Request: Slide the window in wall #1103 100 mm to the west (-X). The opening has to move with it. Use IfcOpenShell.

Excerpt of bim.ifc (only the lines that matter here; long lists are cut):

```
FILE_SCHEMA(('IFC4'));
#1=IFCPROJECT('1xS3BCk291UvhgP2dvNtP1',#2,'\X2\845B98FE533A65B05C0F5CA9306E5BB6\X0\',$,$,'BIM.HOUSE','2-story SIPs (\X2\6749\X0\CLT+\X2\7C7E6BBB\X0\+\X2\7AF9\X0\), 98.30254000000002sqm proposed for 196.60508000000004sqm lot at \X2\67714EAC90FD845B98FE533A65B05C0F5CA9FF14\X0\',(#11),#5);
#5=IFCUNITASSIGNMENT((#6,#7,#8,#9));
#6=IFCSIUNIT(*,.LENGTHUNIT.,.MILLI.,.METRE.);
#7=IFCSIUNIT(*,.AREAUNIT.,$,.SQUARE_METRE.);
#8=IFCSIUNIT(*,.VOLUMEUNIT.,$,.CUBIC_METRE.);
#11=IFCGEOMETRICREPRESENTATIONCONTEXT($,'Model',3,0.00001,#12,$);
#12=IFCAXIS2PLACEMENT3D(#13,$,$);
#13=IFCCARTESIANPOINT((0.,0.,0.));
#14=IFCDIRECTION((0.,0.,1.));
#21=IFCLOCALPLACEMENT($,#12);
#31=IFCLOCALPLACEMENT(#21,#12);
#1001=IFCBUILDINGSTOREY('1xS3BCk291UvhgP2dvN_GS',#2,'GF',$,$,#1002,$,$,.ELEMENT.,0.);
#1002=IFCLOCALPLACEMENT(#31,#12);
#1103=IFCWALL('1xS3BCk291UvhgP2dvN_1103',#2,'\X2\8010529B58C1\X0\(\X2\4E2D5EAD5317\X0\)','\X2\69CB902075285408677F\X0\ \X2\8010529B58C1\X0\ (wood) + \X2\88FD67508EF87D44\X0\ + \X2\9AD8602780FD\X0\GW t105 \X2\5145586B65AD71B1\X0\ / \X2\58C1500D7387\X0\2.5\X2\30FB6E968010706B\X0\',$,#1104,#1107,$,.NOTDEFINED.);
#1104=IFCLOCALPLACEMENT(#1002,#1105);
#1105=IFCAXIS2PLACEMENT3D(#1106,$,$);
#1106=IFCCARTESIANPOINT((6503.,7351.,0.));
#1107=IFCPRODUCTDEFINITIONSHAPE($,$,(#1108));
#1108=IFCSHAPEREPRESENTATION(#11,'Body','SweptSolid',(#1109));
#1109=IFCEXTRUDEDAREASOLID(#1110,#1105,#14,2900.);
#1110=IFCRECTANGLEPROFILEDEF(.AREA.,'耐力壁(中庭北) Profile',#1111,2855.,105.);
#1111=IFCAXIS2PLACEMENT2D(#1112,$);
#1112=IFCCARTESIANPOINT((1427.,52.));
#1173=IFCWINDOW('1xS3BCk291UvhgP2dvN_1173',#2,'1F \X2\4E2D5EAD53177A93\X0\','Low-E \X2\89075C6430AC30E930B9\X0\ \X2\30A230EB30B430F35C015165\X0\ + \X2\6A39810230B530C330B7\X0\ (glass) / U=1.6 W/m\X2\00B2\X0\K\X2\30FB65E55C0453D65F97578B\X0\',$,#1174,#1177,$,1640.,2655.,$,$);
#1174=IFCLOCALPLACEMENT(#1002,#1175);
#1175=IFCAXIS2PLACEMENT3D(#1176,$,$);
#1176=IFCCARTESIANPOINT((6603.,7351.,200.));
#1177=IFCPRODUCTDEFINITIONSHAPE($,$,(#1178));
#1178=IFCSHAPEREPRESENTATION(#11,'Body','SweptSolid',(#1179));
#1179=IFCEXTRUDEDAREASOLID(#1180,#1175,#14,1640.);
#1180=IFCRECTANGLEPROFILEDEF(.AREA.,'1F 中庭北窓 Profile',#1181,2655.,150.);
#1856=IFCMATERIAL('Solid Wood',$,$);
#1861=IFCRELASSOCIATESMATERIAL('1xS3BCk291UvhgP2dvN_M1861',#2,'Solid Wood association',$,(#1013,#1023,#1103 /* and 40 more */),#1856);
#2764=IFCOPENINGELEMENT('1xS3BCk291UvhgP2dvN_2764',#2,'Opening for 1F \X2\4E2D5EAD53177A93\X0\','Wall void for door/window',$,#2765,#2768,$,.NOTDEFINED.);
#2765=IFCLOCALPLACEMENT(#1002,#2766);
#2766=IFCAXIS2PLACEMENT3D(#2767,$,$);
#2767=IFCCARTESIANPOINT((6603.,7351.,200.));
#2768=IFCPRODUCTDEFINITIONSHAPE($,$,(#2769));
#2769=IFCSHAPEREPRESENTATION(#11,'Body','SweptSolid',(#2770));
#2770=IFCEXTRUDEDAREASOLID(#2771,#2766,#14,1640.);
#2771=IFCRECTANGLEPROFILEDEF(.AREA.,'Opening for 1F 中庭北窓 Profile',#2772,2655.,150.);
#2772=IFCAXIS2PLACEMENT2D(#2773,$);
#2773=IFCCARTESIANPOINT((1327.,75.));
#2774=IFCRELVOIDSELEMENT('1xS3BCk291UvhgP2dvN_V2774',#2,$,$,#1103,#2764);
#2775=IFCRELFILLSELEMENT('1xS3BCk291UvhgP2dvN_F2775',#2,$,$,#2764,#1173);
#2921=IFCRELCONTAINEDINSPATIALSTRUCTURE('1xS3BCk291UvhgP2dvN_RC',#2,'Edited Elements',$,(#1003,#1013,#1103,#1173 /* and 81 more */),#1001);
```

```python
import ifcopenshell
import ifcopenshell.api.geometry
import ifcopenshell.util.placement
import ifcopenshell.util.unit

model = ifcopenshell.open("bim.ifc")
unit_scale = ifcopenshell.util.unit.calculate_unit_scale(model)

window = model.by_guid("1xS3BCk291UvhgP2dvN_1173")
opening = window.FillsVoids[0].RelatingOpeningElement
wall = opening.VoidsElements[0].RelatingBuildingElement

wall_matrix = ifcopenshell.util.placement.get_local_placement(wall.ObjectPlacement)
shift = wall_matrix[:3, 0] * -0.1 / unit_scale
before = ifcopenshell.util.placement.get_local_placement(window.ObjectPlacement)[:3, 3].copy()

# The window is not placed relative to its opening, so move both.
for product in (opening, window):
    matrix = ifcopenshell.util.placement.get_local_placement(product.ObjectPlacement)
    matrix[:3, 3] += shift
    ifcopenshell.api.geometry.edit_object_placement(model, product=product, matrix=matrix, is_si=False)

after = ifcopenshell.util.placement.get_local_placement(window.ObjectPlacement)[:3, 3]
print("window moved by", (after - before).round(3) + 0.0)

model.write("bim-out.ifc")
```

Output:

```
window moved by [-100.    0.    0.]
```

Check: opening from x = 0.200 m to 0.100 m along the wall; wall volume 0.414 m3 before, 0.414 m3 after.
